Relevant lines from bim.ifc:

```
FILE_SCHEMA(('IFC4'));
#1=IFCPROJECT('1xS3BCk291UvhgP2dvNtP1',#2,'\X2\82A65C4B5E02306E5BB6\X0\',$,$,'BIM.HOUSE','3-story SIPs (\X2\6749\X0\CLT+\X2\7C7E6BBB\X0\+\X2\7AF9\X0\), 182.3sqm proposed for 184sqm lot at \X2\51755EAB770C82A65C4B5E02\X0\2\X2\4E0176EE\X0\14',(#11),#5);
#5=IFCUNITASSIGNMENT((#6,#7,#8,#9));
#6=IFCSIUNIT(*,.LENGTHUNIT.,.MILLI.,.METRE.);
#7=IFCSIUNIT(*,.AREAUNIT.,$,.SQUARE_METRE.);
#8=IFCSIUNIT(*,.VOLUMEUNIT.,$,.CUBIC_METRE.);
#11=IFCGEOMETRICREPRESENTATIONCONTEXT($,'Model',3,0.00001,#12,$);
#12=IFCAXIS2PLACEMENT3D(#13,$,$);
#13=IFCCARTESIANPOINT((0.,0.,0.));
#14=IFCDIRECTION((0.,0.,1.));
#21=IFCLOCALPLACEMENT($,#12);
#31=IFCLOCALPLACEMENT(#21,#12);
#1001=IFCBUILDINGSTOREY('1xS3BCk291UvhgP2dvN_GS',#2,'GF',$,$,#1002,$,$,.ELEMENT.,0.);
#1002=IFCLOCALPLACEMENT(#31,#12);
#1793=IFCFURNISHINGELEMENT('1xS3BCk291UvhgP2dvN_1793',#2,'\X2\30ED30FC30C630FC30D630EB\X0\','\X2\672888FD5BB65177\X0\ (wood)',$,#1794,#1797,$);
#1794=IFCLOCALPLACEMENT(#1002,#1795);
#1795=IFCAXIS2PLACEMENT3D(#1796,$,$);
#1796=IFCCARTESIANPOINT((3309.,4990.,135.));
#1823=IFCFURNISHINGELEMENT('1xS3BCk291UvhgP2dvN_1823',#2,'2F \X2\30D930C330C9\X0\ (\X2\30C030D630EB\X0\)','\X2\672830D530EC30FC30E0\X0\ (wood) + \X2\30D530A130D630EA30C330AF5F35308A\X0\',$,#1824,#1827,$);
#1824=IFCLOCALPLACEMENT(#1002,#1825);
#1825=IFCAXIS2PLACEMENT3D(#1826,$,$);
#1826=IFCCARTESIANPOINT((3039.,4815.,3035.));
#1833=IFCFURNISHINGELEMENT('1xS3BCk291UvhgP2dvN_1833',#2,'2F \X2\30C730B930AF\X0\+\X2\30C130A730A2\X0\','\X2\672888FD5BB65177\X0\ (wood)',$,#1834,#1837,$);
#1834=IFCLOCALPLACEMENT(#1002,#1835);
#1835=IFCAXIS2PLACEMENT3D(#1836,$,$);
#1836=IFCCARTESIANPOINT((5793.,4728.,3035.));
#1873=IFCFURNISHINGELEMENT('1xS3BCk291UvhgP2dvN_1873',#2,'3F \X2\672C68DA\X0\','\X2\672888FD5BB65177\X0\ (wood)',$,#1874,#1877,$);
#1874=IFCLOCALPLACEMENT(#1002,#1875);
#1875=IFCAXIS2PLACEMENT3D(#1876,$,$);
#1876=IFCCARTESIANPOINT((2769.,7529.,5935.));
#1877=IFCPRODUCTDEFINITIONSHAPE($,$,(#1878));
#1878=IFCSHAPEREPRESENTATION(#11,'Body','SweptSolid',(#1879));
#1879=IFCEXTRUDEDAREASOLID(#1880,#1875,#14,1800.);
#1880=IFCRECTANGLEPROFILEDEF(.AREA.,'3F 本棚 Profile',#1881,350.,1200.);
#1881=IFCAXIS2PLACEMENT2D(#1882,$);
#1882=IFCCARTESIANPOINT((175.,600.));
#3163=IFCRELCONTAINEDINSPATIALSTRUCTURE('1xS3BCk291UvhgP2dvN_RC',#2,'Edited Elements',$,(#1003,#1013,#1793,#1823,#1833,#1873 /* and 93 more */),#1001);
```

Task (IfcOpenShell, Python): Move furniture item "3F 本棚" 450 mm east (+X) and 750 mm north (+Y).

```python
import ifcopenshell
import ifcopenshell.api.geometry
import ifcopenshell.util.placement
import ifcopenshell.util.unit

model = ifcopenshell.open("bim.ifc")
unit_scale = ifcopenshell.util.unit.calculate_unit_scale(model)

item = model.by_guid("1xS3BCk291UvhgP2dvN_1873")
matrix = ifcopenshell.util.placement.get_local_placement(item.ObjectPlacement)
matrix[0, 3] += 0.45 / unit_scale
matrix[1, 3] += 0.75 / unit_scale
ifcopenshell.api.geometry.edit_object_placement(model, product=item, matrix=matrix, is_si=False)

print(ifcopenshell.util.placement.get_local_placement(item.ObjectPlacement).round(3) + 0.0)

model.write("bim_v2.ifc")
```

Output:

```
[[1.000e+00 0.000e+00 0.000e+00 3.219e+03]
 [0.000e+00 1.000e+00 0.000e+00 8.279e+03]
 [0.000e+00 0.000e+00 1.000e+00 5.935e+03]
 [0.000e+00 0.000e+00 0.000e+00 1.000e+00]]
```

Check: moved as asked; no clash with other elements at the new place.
